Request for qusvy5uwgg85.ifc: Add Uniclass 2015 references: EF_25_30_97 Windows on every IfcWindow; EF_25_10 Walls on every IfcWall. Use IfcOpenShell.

First a look at what the model holds.

```python
import ifcopenshell

model = ifcopenshell.open("qusvy5uwgg85.ifc")
print(model.schema)
print("classifications:", [c.Name for c in model.by_type("IfcClassification")])
for ifc_class in ("IfcDoor", "IfcRoof", "IfcStair", "IfcWall", "IfcWindow"):
    print(ifc_class, len(model.by_type(ifc_class)))
```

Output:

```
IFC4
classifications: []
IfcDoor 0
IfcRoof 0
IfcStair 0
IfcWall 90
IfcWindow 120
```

```python
import ifcopenshell
import ifcopenshell.api.classification

model = ifcopenshell.open("qusvy5uwgg85.ifc")

system = ifcopenshell.api.classification.add_classification(model, classification="Uniclass 2015")

codes = {
    "IfcWindow": ("EF_25_30_97", "Windows"),
    "IfcWall": ("EF_25_10", "Walls"),
}
for ifc_class, (code, name) in codes.items():
    products = model.by_type(ifc_class)
    ifcopenshell.api.classification.add_reference(
        model, products=products, classification=system, identification=code, name=name
    )
    print(code, len(products))

model.write("qusvy5uwgg85_v2.ifc")
```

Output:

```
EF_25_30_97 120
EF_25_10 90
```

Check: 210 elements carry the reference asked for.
